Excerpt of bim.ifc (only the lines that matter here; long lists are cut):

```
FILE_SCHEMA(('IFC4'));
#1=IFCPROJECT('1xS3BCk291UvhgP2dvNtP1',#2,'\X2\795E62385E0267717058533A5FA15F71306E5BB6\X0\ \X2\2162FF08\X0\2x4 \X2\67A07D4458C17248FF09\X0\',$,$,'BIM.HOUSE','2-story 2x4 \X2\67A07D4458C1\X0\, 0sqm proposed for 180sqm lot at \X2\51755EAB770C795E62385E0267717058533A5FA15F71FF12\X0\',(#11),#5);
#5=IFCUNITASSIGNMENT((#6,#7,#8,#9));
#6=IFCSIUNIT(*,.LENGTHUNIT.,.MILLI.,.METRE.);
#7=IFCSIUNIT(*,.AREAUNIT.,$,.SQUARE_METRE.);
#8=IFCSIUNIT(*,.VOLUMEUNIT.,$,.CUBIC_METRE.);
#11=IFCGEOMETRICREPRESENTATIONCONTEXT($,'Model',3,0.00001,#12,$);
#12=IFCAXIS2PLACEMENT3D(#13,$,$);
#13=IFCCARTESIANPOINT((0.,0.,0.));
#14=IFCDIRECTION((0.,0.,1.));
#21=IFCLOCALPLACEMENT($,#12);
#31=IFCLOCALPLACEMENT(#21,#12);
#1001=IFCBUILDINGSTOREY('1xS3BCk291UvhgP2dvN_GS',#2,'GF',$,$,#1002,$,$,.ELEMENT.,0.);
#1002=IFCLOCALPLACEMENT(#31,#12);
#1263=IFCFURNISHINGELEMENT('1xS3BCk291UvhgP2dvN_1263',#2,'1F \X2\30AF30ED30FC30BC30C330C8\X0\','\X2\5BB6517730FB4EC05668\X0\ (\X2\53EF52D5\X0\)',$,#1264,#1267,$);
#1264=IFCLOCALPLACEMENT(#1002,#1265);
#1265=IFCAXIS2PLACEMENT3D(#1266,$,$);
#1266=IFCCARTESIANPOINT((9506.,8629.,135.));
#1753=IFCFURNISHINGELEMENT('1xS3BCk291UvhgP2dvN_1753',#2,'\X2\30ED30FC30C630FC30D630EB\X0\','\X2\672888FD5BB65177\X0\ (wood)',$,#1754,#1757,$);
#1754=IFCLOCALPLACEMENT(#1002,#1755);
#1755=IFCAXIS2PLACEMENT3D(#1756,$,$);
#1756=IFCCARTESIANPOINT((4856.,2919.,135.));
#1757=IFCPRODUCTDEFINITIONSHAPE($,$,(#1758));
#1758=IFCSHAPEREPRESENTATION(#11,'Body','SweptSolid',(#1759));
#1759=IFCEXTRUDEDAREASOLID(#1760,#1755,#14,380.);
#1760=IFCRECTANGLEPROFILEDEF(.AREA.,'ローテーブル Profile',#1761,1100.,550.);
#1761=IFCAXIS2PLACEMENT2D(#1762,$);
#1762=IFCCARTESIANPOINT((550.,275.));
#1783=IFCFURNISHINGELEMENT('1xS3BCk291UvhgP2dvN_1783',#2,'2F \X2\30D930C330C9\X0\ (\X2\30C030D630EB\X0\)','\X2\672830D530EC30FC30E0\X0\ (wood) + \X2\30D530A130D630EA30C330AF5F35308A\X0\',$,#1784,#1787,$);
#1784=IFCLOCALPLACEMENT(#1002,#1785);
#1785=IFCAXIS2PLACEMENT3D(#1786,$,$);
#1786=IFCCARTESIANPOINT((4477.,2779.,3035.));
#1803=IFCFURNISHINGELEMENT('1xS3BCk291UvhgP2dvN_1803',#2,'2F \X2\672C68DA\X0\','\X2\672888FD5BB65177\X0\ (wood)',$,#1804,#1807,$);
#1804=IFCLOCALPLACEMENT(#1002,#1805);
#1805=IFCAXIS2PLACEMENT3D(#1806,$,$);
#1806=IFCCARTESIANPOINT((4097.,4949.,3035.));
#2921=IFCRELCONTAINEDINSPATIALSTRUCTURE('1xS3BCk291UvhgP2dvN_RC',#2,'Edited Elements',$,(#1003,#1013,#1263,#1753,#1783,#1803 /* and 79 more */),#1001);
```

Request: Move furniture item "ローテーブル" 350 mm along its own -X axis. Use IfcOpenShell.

```python
import ifcopenshell
import ifcopenshell.api.geometry
import ifcopenshell.util.placement
import ifcopenshell.util.unit

model = ifcopenshell.open("bim.ifc")
unit_scale = ifcopenshell.util.unit.calculate_unit_scale(model)

item = model.by_guid("1xS3BCk291UvhgP2dvN_1753")
matrix = ifcopenshell.util.placement.get_local_placement(item.ObjectPlacement)
matrix[:3, 3] -= matrix[:3, 0] * 0.35 / unit_scale
ifcopenshell.api.geometry.edit_object_placement(model, product=item, matrix=matrix, is_si=False)

print(ifcopenshell.util.placement.get_local_placement(item.ObjectPlacement).round(3) + 0.0)

model.write("bim_updated.ifc")
```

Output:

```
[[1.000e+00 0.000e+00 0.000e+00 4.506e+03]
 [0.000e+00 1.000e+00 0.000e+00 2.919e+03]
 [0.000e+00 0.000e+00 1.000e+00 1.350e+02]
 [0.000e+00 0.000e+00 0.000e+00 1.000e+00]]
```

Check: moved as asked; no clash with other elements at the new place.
